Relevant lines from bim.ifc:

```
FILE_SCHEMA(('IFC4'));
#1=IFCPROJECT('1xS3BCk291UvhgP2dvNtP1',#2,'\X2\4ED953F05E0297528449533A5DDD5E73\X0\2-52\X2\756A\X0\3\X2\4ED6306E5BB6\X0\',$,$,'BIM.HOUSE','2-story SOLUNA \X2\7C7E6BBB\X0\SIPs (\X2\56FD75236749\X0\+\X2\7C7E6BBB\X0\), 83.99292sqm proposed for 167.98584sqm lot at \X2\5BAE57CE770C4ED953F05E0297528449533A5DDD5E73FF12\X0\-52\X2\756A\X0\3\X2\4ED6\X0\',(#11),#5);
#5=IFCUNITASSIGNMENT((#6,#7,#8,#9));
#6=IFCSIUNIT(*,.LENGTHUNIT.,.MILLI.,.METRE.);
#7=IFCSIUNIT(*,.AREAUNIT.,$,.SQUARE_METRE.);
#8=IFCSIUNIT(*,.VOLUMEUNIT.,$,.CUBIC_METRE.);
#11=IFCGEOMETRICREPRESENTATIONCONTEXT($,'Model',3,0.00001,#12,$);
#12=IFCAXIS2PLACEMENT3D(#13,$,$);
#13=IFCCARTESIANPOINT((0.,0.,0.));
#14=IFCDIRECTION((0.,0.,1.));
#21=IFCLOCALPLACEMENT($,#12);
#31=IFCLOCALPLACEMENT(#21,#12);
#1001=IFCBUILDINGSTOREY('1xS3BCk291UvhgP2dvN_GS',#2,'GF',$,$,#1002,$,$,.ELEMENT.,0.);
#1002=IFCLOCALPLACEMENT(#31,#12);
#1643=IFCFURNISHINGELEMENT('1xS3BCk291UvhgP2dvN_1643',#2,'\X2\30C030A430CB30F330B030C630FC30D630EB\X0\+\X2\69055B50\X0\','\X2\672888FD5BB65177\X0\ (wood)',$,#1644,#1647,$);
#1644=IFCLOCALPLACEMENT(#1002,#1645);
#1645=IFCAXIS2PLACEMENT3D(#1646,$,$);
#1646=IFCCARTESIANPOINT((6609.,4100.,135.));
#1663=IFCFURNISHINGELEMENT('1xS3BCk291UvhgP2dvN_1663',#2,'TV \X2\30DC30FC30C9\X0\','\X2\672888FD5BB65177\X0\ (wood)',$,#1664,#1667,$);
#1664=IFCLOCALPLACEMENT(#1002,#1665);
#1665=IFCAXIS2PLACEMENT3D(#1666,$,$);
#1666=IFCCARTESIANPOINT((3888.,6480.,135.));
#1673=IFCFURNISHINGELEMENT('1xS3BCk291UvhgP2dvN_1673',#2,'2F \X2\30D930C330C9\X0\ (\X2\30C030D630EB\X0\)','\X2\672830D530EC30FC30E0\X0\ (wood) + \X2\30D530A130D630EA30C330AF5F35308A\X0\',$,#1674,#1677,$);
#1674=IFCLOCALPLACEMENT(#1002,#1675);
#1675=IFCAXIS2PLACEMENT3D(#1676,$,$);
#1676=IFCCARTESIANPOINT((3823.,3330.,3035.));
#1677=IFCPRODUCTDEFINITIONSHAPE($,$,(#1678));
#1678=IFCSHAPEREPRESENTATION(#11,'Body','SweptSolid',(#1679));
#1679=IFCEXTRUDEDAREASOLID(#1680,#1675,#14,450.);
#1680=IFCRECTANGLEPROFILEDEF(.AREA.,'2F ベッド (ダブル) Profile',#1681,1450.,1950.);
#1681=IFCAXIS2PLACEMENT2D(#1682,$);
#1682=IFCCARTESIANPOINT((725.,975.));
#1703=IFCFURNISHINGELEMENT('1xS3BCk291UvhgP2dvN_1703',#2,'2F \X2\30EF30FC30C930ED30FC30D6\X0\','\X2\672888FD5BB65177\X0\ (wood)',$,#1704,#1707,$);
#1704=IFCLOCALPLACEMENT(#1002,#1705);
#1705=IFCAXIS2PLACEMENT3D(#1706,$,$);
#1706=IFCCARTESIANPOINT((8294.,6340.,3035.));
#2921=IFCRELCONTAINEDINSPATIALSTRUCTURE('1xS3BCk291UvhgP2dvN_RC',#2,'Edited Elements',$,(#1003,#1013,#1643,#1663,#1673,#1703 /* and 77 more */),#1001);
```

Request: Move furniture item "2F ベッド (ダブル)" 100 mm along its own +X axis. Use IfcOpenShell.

```python
import ifcopenshell
import ifcopenshell.api.geometry
import ifcopenshell.util.placement
import ifcopenshell.util.unit

model = ifcopenshell.open("bim.ifc")
unit_scale = ifcopenshell.util.unit.calculate_unit_scale(model)

item = model.by_guid("1xS3BCk291UvhgP2dvN_1673")
matrix = ifcopenshell.util.placement.get_local_placement(item.ObjectPlacement)
matrix[:3, 3] += matrix[:3, 0] * 0.1 / unit_scale
ifcopenshell.api.geometry.edit_object_placement(model, product=item, matrix=matrix, is_si=False)

print(ifcopenshell.util.placement.get_local_placement(item.ObjectPlacement).round(3) + 0.0)

model.write("bim-out.ifc")
```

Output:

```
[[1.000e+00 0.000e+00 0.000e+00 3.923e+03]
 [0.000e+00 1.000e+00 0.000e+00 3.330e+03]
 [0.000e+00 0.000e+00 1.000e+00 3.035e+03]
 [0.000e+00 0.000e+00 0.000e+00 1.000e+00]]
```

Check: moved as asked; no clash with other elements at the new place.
